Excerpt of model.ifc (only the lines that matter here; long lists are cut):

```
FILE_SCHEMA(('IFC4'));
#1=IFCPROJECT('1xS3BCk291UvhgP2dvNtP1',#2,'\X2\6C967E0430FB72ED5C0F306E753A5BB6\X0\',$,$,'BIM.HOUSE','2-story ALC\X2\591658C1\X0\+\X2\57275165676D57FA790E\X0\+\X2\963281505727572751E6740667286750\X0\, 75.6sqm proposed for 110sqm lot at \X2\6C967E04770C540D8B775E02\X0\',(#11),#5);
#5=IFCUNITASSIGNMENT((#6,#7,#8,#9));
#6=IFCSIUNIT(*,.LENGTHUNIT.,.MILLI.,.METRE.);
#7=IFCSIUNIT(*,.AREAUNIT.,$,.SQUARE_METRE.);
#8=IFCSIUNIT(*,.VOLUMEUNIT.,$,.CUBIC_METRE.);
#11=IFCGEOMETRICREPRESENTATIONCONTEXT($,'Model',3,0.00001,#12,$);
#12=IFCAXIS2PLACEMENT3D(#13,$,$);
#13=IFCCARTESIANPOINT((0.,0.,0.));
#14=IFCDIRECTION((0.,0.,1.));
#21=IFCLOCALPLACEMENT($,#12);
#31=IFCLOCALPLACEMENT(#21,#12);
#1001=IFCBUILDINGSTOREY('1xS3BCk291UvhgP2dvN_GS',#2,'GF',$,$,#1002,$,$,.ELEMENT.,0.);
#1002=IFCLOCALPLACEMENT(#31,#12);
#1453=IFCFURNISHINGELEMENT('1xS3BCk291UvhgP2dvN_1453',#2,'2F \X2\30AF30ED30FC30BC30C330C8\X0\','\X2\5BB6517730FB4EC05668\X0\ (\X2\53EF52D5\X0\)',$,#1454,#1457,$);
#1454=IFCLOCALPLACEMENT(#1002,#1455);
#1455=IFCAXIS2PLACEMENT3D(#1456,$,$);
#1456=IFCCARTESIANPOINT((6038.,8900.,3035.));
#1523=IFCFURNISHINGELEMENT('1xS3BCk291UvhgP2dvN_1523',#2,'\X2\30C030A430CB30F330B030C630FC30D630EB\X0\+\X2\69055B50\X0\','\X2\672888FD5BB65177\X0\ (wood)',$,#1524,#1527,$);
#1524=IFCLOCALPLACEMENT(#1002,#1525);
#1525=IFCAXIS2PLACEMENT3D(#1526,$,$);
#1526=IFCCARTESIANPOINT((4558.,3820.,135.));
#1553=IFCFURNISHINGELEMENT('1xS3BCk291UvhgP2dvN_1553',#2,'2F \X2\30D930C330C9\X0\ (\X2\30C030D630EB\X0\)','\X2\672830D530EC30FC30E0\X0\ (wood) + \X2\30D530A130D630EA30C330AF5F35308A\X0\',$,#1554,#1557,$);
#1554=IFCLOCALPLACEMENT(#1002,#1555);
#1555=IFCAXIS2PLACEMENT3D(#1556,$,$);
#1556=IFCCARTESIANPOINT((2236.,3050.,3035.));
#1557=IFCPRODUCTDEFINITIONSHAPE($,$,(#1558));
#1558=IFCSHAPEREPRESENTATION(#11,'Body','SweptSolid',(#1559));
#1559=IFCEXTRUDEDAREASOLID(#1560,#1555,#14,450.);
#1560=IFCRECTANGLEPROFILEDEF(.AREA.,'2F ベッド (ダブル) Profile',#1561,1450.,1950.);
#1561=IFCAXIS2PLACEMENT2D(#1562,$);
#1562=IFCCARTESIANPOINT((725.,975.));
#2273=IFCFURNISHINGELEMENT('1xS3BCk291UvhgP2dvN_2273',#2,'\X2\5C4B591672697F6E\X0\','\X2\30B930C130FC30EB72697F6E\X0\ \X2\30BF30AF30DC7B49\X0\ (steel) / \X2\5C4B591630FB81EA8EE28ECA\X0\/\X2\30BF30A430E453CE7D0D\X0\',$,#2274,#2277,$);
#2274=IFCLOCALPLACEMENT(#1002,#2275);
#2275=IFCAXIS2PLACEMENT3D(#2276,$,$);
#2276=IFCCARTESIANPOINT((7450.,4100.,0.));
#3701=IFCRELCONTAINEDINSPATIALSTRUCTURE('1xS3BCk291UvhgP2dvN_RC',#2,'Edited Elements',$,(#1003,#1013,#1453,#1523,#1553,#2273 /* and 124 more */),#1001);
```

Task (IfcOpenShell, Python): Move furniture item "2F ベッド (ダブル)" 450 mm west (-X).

```python
import ifcopenshell
import ifcopenshell.api.geometry
import ifcopenshell.util.placement

model = ifcopenshell.open("model.ifc")

item = model.by_guid("1xS3BCk291UvhgP2dvN_1553")
matrix = ifcopenshell.util.placement.get_local_placement(item.ObjectPlacement)
matrix[0, 3] -= 450.0
ifcopenshell.api.geometry.edit_object_placement(model, product=item, matrix=matrix, is_si=False)

print(ifcopenshell.util.placement.get_local_placement(item.ObjectPlacement).round(3) + 0.0)

model.write("model_v2.ifc")
```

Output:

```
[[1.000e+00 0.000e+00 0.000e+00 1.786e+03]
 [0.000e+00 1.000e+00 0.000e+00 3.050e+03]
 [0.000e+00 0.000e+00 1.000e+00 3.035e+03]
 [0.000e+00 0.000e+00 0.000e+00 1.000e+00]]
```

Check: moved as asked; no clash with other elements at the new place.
